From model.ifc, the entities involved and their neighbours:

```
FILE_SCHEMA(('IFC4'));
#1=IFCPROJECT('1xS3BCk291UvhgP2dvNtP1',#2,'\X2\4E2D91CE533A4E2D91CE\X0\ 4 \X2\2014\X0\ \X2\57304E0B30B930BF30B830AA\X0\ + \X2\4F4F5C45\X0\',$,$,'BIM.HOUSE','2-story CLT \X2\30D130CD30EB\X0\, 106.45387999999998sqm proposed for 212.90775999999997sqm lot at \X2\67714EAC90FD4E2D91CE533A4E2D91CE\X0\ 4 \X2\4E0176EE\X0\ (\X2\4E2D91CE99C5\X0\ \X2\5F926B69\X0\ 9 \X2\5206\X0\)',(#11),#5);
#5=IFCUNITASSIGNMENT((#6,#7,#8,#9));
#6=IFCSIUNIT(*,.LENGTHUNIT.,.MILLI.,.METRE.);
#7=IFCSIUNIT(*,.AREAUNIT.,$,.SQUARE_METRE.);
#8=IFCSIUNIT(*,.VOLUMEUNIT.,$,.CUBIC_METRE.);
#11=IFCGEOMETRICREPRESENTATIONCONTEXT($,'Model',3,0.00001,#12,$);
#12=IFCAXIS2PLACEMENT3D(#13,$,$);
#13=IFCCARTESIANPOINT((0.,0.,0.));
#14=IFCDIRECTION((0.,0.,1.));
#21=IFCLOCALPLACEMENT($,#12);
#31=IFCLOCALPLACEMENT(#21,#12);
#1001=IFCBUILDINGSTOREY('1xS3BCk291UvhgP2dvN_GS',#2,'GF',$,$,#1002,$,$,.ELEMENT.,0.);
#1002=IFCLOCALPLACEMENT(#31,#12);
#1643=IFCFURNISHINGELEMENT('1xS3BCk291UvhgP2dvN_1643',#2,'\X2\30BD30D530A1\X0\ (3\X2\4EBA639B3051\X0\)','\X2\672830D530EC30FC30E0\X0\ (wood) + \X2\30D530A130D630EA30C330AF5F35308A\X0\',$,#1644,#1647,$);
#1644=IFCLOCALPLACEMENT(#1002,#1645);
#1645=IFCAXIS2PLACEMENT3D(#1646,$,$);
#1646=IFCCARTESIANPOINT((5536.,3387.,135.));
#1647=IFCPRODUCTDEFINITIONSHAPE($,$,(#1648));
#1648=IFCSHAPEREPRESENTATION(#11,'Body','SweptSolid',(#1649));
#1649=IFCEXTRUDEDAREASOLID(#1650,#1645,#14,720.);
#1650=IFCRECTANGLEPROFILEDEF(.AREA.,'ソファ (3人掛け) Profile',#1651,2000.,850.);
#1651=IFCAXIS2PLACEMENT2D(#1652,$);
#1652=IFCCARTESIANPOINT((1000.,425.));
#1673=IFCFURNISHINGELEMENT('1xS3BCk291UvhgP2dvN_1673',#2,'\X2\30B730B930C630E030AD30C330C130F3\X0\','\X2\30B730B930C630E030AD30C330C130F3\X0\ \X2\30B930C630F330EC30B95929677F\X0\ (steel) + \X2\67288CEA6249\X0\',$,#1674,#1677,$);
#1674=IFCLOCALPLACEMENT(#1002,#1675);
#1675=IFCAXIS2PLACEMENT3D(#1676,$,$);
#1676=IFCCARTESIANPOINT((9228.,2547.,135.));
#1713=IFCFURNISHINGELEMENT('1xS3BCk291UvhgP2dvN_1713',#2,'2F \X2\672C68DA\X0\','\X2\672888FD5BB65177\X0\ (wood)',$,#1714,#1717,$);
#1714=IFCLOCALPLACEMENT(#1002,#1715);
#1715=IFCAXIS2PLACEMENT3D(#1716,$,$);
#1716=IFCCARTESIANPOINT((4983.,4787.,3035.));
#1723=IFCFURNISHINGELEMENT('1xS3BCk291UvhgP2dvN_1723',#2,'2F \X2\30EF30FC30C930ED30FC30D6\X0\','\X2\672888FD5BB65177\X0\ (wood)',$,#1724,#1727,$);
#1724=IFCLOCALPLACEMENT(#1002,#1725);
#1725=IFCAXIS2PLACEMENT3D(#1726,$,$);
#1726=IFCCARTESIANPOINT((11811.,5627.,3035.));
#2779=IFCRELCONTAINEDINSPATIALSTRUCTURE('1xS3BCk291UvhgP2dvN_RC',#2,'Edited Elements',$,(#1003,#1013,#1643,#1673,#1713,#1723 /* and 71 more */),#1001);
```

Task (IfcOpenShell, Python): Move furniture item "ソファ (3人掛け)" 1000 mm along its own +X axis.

```python
import ifcopenshell
import ifcopenshell.api.geometry
import ifcopenshell.util.placement
import ifcopenshell.util.unit

model = ifcopenshell.open("model.ifc")
unit_scale = ifcopenshell.util.unit.calculate_unit_scale(model)

item = model.by_guid("1xS3BCk291UvhgP2dvN_1643")
matrix = ifcopenshell.util.placement.get_local_placement(item.ObjectPlacement)
matrix[:3, 3] += matrix[:3, 0] * 1 / unit_scale
ifcopenshell.api.geometry.edit_object_placement(model, product=item, matrix=matrix, is_si=False)

print(ifcopenshell.util.placement.get_local_placement(item.ObjectPlacement).round(3) + 0.0)

model.write("model_rev.ifc")
```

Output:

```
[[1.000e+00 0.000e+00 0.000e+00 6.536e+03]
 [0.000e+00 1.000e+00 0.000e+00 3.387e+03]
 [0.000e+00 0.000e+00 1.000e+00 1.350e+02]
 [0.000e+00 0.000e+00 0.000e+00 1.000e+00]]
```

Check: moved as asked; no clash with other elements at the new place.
